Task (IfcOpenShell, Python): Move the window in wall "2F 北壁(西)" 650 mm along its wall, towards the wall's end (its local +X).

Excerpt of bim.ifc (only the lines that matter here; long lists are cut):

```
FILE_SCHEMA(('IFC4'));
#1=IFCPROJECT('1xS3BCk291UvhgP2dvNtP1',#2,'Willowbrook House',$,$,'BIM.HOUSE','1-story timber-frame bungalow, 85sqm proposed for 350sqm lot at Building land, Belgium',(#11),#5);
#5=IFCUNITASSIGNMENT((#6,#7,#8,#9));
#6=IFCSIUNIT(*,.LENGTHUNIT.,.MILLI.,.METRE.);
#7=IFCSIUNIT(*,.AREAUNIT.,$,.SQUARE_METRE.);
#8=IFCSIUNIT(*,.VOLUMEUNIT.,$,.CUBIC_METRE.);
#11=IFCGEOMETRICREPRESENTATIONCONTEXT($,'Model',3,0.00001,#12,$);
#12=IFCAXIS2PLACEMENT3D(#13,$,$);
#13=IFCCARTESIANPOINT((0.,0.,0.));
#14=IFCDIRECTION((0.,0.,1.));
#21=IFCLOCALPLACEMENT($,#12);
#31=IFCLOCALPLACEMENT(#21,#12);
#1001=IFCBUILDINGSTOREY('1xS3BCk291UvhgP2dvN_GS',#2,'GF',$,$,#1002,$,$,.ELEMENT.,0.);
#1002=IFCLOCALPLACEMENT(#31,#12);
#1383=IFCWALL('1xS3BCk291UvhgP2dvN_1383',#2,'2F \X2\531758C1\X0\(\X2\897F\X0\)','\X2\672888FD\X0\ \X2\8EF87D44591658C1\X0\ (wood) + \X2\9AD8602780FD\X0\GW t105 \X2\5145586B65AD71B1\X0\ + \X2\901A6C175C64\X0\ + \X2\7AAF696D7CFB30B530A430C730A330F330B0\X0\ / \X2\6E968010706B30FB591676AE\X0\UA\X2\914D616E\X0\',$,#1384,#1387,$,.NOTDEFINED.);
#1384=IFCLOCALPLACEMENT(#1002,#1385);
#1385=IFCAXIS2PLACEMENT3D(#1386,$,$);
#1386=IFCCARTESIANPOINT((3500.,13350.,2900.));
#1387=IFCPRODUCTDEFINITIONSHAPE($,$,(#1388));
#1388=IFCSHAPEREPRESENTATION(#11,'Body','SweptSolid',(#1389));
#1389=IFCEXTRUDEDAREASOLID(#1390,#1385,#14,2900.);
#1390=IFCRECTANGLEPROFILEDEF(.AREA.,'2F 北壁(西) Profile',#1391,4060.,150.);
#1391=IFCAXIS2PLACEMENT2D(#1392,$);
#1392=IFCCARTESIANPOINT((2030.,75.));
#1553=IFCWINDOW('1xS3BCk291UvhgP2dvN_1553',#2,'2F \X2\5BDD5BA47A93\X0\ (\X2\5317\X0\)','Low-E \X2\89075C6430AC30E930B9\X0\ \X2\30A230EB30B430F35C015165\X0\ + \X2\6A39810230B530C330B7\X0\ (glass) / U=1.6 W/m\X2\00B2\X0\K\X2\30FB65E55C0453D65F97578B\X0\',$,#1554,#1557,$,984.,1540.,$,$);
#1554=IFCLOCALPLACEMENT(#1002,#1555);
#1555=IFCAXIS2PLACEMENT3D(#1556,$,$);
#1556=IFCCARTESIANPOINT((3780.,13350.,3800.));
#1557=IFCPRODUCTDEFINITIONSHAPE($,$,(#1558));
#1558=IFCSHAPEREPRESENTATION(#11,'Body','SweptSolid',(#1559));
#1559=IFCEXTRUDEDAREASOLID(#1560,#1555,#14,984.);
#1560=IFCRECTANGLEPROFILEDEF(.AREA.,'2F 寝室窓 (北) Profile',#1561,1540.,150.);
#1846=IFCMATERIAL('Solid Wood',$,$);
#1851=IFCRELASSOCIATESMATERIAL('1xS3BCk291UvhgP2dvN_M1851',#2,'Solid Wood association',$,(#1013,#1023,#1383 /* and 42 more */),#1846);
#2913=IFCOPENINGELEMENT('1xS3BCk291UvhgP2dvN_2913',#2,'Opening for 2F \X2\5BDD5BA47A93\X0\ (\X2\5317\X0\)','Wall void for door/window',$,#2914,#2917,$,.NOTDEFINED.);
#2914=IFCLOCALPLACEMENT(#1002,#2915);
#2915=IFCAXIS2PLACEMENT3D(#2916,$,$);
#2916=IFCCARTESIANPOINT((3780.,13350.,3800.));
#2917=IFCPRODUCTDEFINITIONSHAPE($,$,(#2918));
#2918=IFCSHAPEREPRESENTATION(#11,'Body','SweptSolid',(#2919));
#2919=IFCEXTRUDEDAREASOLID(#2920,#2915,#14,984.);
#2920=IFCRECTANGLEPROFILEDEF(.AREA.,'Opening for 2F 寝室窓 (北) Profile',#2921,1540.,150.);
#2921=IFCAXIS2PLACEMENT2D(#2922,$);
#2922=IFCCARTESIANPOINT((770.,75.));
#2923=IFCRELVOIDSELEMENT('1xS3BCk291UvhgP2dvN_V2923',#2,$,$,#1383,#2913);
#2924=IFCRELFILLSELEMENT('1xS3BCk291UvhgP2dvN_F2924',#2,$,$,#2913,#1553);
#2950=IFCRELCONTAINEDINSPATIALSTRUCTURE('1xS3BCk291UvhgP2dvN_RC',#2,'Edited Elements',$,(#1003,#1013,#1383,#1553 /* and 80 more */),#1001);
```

```python
import ifcopenshell
import ifcopenshell.api.geometry
import ifcopenshell.util.placement

model = ifcopenshell.open("bim.ifc")

window = model.by_guid("1xS3BCk291UvhgP2dvN_1553")
opening = window.FillsVoids[0].RelatingOpeningElement
wall = opening.VoidsElements[0].RelatingBuildingElement

wall_matrix = ifcopenshell.util.placement.get_local_placement(wall.ObjectPlacement)
shift = wall_matrix[:3, 0] * 650.0
before = ifcopenshell.util.placement.get_local_placement(window.ObjectPlacement)[:3, 3].copy()

# The window is not placed relative to its opening, so move both.
for product in (opening, window):
    matrix = ifcopenshell.util.placement.get_local_placement(product.ObjectPlacement)
    matrix[:3, 3] += shift
    ifcopenshell.api.geometry.edit_object_placement(model, product=product, matrix=matrix, is_si=False)

after = ifcopenshell.util.placement.get_local_placement(window.ObjectPlacement)[:3, 3]
print("window moved by", (after - before).round(3) + 0.0)

model.write("bim-out.ifc")
```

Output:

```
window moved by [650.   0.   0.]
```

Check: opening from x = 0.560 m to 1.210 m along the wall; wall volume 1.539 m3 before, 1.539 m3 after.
